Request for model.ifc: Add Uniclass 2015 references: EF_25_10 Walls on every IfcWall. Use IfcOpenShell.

First a look at what the model holds.

```python
import ifcopenshell

model = ifcopenshell.open("model.ifc")
print(model.schema)
print("classifications:", [c.Name for c in model.by_type("IfcClassification")])
for ifc_class in ("IfcDoor", "IfcRoof", "IfcStair", "IfcWall", "IfcWindow"):
    print(ifc_class, len(model.by_type(ifc_class)))
```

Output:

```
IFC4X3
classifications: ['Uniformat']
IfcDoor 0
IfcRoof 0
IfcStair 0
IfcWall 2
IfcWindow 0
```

```python
import ifcopenshell
import ifcopenshell.api.classification

model = ifcopenshell.open("model.ifc")

system = ifcopenshell.api.classification.add_classification(model, classification="Uniclass 2015")

codes = {
    "IfcWall": ("EF_25_10", "Walls"),
}
for ifc_class, (code, name) in codes.items():
    products = model.by_type(ifc_class)
    ifcopenshell.api.classification.add_reference(
        model, products=products, classification=system, identification=code, name=name
    )
    print(code, len(products))

model.write("model-out.ifc")
```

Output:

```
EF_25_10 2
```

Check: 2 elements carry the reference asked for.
